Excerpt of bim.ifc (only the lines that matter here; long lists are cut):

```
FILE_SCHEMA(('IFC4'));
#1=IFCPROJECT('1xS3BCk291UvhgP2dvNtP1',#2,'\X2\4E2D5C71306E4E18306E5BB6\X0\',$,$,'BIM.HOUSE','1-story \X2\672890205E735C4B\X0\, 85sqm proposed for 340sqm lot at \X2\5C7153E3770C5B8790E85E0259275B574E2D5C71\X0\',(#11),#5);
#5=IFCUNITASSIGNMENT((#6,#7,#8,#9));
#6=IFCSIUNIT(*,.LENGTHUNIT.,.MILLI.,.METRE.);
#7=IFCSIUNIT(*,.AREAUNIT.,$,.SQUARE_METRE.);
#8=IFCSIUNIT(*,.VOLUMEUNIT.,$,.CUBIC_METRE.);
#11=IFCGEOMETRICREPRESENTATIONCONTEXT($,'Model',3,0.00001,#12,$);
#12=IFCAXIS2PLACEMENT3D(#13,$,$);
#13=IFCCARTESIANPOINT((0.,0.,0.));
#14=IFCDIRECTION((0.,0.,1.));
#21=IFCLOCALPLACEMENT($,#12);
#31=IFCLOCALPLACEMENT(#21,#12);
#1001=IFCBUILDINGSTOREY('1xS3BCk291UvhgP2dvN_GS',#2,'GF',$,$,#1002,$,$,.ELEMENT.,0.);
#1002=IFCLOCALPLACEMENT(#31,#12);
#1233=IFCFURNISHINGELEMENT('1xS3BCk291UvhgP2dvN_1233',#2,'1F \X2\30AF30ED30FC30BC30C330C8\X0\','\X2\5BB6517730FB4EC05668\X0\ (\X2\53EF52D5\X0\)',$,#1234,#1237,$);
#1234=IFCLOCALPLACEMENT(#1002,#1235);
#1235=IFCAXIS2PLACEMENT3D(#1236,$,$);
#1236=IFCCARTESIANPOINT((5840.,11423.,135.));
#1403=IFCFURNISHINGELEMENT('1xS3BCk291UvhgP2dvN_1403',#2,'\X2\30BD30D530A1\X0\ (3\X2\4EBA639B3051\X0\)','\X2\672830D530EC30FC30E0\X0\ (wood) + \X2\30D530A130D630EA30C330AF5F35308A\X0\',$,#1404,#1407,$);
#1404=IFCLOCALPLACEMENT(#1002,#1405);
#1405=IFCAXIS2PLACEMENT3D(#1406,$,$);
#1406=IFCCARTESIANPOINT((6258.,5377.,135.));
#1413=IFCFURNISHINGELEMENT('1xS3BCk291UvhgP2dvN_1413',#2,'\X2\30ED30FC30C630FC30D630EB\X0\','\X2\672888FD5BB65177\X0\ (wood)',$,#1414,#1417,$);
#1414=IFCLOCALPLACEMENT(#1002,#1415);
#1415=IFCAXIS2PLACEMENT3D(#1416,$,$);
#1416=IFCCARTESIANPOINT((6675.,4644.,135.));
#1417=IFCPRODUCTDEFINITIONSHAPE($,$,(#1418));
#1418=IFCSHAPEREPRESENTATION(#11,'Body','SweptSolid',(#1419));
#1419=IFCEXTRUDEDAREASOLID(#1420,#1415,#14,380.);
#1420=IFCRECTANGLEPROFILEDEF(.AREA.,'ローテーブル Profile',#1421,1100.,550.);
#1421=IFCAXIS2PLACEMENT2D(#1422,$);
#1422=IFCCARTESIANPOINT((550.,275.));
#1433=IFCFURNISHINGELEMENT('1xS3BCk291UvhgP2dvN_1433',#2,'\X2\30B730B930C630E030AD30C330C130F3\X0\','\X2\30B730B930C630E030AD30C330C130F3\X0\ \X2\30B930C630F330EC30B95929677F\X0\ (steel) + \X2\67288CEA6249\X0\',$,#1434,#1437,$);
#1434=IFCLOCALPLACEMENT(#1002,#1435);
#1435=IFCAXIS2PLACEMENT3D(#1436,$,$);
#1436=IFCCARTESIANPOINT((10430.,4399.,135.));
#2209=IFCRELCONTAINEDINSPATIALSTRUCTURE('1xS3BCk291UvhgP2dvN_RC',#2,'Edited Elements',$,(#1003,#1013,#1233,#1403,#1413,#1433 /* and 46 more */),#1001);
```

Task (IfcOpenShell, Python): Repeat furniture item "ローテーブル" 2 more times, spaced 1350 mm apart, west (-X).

```python
import numpy as np
import ifcopenshell
import ifcopenshell.api.geometry
import ifcopenshell.api.root
import ifcopenshell.util.element
import ifcopenshell.util.placement
import ifcopenshell.util.unit

model = ifcopenshell.open("bim.ifc")
unit_scale = ifcopenshell.util.unit.calculate_unit_scale(model)


def reuse_history(source, copy):
    """copy_class also copies each property set's owner history, people and application; keep the originals."""
    for rel in copy.IsDefinedBy:
        if rel.is_a("IfcRelDefinesByProperties") and (history := rel.RelatingPropertyDefinition.OwnerHistory):
            rel.RelatingPropertyDefinition.OwnerHistory = source.OwnerHistory
            ifcopenshell.util.element.remove_deep2(model, history)


source = model.by_id(1413)
base = ifcopenshell.util.placement.get_local_placement(source.ObjectPlacement)
step = np.array([-1.0, 0.0, 0.0]) * 1.35 / unit_scale

for i in range(1, 3):
    copy = ifcopenshell.api.root.copy_class(model, product=source)
    copy.Representation = ifcopenshell.util.element.copy_deep(
        model, source.Representation, exclude=["IfcGeometricRepresentationContext", "IfcRepresentationMap"]
    )
    reuse_history(source, copy)
    matrix = base.copy()
    matrix[:3, 3] += i * step
    print("added at", matrix[:3, 3].round(3) + 0.0)
    ifcopenshell.api.geometry.edit_object_placement(model, product=copy, matrix=matrix, is_si=False)

model.write("bim_edited.ifc")
```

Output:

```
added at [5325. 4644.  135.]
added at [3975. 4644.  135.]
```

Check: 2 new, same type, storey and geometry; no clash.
